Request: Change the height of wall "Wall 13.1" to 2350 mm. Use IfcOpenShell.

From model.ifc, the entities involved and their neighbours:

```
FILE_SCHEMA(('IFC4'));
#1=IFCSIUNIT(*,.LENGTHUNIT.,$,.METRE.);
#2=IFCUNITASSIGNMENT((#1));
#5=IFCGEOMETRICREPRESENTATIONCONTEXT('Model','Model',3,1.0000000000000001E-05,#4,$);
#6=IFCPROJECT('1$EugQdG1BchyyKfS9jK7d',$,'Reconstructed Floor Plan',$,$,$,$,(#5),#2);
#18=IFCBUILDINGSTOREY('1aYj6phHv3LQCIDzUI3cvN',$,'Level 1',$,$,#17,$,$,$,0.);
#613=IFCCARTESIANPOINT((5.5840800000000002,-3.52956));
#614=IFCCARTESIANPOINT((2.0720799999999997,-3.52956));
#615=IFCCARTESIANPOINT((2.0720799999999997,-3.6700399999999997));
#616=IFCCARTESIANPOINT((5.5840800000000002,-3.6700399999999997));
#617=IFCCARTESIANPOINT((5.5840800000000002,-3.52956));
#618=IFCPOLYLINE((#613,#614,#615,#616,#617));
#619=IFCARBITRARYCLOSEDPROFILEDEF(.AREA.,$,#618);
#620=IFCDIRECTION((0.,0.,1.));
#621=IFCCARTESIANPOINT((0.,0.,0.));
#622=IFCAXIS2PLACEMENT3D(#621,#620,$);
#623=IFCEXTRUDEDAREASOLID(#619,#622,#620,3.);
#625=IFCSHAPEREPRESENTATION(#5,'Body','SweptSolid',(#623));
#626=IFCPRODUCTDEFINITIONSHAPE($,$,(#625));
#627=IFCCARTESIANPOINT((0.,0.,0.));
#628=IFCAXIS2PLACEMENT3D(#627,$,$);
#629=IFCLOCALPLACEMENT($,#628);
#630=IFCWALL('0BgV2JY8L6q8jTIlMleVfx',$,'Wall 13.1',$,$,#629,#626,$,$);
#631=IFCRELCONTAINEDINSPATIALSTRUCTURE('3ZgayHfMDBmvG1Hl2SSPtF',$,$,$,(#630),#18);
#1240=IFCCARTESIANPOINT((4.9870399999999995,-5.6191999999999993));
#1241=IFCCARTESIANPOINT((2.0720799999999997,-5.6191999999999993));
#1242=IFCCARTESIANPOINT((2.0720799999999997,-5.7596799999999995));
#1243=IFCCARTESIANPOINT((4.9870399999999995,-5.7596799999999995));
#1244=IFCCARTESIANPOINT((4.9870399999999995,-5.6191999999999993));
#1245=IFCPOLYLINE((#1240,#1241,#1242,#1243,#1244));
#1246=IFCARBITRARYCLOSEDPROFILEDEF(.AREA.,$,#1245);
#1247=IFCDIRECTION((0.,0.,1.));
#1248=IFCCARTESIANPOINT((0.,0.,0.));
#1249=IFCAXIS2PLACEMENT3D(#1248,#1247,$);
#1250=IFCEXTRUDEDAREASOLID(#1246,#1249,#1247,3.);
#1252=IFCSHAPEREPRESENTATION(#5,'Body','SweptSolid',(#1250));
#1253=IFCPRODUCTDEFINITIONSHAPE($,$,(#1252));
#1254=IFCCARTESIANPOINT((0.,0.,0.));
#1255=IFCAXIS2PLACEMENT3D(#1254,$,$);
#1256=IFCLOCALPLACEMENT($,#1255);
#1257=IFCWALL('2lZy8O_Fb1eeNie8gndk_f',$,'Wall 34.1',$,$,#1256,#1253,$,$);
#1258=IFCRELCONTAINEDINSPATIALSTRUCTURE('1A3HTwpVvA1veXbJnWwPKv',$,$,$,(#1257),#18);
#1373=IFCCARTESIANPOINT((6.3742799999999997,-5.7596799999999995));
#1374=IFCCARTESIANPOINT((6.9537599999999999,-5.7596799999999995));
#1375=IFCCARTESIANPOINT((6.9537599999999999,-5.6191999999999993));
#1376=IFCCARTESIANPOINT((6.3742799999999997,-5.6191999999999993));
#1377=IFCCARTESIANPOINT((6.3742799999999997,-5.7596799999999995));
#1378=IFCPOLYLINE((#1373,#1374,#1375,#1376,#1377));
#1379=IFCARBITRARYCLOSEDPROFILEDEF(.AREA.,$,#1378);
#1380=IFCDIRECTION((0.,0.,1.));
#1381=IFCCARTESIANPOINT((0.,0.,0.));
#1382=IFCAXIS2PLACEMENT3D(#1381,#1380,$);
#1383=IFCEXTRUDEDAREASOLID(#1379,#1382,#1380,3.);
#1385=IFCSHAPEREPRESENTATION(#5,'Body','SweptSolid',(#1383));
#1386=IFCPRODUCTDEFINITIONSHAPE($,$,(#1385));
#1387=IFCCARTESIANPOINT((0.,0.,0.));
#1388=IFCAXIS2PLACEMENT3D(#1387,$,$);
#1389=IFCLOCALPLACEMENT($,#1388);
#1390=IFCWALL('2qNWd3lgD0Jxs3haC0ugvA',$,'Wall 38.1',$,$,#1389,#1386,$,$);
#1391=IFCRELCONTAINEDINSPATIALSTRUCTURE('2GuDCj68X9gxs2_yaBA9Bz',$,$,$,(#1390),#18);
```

```python
import ifcopenshell
import ifcopenshell.geom
import ifcopenshell.util.shape
import ifcopenshell.util.unit

model = ifcopenshell.open("model.ifc")
unit_scale = ifcopenshell.util.unit.calculate_unit_scale(model)
settings = ifcopenshell.geom.settings()


def volume(element):
    """Net volume in cubic metres, openings subtracted."""
    shape = ifcopenshell.geom.create_shape(settings, element)
    return ifcopenshell.util.shape.get_volume(shape.geometry)


wall = model.by_guid("0BgV2JY8L6q8jTIlMleVfx")
before = volume(wall)

body = next(r for r in wall.Representation.Representations if r.RepresentationIdentifier == "Body")
solid = body.Items[0]
old_height = solid.Depth
solid.Depth = 2.35 / unit_scale
after = volume(wall)

print(f"height {old_height:g} -> {solid.Depth:g}, volume {before:.3f} -> {after:.3f} m3")

model.write("model_updated.ifc")
```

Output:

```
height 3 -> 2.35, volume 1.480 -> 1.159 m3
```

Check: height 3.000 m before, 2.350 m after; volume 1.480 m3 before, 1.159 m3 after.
